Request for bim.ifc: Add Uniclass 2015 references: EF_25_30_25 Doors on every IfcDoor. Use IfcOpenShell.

First a look at what the model holds.

```python
import ifcopenshell

model = ifcopenshell.open("bim.ifc")
print(model.schema)
print("classifications:", [c.Name for c in model.by_type("IfcClassification")])
for ifc_class in ("IfcDoor", "IfcRoof", "IfcStair", "IfcWall", "IfcWindow"):
    print(ifc_class, len(model.by_type(ifc_class)))
```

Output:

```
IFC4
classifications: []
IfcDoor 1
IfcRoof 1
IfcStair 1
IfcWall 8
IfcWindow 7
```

```python
import ifcopenshell
import ifcopenshell.api.classification

model = ifcopenshell.open("bim.ifc")

system = ifcopenshell.api.classification.add_classification(model, classification="Uniclass 2015")

codes = {
    "IfcDoor": ("EF_25_30_25", "Doors"),
}
for ifc_class, (code, name) in codes.items():
    products = model.by_type(ifc_class)
    ifcopenshell.api.classification.add_reference(
        model, products=products, classification=system, identification=code, name=name
    )
    print(code, len(products))

model.write("bim_v2.ifc")
```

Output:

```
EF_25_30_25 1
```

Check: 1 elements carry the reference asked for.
